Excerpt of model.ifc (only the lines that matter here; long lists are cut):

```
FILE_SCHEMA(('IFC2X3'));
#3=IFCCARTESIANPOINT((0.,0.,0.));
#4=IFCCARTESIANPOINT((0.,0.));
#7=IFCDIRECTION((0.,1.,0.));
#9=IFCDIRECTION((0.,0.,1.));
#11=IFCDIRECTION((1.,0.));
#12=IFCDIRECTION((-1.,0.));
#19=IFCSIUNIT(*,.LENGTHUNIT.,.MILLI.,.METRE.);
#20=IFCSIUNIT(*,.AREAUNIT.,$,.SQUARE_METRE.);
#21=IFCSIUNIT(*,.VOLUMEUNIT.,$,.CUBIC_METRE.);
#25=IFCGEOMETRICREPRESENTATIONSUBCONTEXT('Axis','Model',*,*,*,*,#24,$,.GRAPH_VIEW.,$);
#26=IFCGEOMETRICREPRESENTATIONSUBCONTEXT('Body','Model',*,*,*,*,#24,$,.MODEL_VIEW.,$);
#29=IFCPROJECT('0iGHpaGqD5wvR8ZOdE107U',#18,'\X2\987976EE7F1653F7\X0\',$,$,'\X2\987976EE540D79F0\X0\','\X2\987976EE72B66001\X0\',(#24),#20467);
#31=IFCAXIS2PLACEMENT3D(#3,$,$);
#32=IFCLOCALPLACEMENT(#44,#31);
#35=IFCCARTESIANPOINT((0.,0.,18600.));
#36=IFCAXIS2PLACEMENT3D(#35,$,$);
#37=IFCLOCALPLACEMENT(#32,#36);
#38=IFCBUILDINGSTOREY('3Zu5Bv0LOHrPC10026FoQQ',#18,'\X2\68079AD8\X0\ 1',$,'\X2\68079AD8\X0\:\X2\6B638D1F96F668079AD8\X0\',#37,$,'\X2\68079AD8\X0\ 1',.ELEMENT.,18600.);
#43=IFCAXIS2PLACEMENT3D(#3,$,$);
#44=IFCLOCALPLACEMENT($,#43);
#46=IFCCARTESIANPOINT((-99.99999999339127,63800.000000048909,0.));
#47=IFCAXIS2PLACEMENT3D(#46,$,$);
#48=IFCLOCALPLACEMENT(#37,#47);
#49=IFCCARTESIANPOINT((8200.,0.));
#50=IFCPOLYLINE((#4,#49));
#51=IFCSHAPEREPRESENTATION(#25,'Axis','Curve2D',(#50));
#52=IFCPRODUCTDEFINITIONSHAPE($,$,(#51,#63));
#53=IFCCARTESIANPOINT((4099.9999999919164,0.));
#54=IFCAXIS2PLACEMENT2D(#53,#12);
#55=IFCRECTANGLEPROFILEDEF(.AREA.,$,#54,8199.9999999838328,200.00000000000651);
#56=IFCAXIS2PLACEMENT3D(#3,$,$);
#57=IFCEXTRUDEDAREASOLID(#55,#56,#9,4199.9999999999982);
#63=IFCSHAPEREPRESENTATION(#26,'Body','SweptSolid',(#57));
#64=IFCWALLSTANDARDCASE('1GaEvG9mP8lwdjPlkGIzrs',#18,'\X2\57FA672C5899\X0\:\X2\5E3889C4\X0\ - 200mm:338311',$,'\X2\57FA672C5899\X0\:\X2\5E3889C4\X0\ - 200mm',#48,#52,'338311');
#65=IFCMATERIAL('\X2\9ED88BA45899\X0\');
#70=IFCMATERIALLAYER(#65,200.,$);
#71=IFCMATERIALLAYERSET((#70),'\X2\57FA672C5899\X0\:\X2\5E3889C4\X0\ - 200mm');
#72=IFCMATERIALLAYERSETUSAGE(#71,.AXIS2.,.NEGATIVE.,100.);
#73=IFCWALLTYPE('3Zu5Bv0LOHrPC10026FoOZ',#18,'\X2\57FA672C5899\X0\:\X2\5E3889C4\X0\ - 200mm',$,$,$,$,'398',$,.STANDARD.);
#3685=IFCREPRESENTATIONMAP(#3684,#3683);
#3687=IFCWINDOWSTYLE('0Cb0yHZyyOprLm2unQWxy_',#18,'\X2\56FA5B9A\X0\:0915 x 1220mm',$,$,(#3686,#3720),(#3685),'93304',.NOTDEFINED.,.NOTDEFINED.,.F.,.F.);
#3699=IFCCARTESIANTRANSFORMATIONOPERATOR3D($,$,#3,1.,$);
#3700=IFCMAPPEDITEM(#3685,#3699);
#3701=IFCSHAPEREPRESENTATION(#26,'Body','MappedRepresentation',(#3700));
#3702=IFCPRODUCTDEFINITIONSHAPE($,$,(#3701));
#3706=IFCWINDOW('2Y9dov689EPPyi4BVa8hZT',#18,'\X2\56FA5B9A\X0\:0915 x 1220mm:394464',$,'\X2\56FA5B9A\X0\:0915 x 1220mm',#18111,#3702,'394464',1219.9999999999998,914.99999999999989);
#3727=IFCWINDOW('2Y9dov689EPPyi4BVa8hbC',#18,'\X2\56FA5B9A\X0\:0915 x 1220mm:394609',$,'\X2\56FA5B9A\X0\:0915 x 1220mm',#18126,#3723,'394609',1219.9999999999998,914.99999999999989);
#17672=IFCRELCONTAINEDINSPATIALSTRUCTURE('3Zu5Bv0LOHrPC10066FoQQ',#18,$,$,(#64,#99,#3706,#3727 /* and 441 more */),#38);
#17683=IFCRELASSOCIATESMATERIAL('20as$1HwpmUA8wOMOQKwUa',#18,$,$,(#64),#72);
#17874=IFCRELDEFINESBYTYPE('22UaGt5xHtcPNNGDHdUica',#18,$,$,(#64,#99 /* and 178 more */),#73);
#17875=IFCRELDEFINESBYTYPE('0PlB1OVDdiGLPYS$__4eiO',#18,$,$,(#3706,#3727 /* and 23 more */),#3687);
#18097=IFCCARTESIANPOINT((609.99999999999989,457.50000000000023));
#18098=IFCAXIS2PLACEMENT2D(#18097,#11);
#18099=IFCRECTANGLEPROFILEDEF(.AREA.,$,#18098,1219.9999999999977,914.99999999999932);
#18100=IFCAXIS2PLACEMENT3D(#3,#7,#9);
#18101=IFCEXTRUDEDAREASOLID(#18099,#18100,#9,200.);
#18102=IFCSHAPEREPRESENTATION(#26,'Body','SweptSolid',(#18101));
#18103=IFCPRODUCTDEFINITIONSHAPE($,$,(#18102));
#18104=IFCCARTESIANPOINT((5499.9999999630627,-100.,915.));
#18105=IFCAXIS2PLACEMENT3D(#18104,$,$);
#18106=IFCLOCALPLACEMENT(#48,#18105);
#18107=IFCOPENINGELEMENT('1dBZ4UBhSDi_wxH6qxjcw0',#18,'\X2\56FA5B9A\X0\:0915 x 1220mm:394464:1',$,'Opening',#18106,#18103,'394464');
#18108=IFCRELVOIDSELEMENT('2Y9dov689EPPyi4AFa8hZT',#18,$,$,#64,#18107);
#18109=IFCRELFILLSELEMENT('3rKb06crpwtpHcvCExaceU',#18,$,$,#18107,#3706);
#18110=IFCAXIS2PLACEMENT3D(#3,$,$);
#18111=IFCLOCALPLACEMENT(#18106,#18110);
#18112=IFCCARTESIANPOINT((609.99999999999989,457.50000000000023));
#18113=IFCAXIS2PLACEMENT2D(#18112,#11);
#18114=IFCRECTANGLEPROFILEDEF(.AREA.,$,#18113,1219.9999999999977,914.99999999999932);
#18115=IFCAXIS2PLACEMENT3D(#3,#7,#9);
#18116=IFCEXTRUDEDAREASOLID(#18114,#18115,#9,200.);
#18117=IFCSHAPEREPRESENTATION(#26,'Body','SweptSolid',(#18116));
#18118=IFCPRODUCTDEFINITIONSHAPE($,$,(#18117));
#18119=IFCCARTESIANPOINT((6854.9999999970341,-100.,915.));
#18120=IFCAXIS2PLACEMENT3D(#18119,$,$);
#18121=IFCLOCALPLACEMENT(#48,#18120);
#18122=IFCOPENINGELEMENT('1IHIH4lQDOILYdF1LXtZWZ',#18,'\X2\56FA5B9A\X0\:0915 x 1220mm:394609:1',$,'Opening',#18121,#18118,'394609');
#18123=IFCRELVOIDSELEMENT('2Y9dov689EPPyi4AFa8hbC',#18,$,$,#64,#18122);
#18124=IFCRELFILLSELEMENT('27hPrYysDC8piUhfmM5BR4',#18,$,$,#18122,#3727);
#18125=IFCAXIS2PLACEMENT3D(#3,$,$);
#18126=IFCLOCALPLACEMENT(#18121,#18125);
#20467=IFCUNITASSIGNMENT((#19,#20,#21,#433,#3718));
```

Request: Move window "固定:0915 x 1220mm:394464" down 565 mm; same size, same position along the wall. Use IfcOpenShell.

```python
import numpy as np
import ifcopenshell
import ifcopenshell.api.geometry
import ifcopenshell.util.placement
import ifcopenshell.util.unit

model = ifcopenshell.open("model.ifc")
unit_scale = ifcopenshell.util.unit.calculate_unit_scale(model)

window = model.by_guid("2Y9dov689EPPyi4BVa8hZT")
opening = window.FillsVoids[0].RelatingOpeningElement
dz = -0.565 / unit_scale

shift = np.array([0.0, 0.0, dz])
# The window is placed relative to its opening, so it follows when the opening moves.
matrix = ifcopenshell.util.placement.get_local_placement(opening.ObjectPlacement)
matrix[:3, 3] += shift
ifcopenshell.api.geometry.edit_object_placement(
    model, product=opening, matrix=matrix, is_si=False, should_transform_children=True
)

print(f"moved by {dz * unit_scale:+.3f} m")

model.write("model_rev.ifc")
```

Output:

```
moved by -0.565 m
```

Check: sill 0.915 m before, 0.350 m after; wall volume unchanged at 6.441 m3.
